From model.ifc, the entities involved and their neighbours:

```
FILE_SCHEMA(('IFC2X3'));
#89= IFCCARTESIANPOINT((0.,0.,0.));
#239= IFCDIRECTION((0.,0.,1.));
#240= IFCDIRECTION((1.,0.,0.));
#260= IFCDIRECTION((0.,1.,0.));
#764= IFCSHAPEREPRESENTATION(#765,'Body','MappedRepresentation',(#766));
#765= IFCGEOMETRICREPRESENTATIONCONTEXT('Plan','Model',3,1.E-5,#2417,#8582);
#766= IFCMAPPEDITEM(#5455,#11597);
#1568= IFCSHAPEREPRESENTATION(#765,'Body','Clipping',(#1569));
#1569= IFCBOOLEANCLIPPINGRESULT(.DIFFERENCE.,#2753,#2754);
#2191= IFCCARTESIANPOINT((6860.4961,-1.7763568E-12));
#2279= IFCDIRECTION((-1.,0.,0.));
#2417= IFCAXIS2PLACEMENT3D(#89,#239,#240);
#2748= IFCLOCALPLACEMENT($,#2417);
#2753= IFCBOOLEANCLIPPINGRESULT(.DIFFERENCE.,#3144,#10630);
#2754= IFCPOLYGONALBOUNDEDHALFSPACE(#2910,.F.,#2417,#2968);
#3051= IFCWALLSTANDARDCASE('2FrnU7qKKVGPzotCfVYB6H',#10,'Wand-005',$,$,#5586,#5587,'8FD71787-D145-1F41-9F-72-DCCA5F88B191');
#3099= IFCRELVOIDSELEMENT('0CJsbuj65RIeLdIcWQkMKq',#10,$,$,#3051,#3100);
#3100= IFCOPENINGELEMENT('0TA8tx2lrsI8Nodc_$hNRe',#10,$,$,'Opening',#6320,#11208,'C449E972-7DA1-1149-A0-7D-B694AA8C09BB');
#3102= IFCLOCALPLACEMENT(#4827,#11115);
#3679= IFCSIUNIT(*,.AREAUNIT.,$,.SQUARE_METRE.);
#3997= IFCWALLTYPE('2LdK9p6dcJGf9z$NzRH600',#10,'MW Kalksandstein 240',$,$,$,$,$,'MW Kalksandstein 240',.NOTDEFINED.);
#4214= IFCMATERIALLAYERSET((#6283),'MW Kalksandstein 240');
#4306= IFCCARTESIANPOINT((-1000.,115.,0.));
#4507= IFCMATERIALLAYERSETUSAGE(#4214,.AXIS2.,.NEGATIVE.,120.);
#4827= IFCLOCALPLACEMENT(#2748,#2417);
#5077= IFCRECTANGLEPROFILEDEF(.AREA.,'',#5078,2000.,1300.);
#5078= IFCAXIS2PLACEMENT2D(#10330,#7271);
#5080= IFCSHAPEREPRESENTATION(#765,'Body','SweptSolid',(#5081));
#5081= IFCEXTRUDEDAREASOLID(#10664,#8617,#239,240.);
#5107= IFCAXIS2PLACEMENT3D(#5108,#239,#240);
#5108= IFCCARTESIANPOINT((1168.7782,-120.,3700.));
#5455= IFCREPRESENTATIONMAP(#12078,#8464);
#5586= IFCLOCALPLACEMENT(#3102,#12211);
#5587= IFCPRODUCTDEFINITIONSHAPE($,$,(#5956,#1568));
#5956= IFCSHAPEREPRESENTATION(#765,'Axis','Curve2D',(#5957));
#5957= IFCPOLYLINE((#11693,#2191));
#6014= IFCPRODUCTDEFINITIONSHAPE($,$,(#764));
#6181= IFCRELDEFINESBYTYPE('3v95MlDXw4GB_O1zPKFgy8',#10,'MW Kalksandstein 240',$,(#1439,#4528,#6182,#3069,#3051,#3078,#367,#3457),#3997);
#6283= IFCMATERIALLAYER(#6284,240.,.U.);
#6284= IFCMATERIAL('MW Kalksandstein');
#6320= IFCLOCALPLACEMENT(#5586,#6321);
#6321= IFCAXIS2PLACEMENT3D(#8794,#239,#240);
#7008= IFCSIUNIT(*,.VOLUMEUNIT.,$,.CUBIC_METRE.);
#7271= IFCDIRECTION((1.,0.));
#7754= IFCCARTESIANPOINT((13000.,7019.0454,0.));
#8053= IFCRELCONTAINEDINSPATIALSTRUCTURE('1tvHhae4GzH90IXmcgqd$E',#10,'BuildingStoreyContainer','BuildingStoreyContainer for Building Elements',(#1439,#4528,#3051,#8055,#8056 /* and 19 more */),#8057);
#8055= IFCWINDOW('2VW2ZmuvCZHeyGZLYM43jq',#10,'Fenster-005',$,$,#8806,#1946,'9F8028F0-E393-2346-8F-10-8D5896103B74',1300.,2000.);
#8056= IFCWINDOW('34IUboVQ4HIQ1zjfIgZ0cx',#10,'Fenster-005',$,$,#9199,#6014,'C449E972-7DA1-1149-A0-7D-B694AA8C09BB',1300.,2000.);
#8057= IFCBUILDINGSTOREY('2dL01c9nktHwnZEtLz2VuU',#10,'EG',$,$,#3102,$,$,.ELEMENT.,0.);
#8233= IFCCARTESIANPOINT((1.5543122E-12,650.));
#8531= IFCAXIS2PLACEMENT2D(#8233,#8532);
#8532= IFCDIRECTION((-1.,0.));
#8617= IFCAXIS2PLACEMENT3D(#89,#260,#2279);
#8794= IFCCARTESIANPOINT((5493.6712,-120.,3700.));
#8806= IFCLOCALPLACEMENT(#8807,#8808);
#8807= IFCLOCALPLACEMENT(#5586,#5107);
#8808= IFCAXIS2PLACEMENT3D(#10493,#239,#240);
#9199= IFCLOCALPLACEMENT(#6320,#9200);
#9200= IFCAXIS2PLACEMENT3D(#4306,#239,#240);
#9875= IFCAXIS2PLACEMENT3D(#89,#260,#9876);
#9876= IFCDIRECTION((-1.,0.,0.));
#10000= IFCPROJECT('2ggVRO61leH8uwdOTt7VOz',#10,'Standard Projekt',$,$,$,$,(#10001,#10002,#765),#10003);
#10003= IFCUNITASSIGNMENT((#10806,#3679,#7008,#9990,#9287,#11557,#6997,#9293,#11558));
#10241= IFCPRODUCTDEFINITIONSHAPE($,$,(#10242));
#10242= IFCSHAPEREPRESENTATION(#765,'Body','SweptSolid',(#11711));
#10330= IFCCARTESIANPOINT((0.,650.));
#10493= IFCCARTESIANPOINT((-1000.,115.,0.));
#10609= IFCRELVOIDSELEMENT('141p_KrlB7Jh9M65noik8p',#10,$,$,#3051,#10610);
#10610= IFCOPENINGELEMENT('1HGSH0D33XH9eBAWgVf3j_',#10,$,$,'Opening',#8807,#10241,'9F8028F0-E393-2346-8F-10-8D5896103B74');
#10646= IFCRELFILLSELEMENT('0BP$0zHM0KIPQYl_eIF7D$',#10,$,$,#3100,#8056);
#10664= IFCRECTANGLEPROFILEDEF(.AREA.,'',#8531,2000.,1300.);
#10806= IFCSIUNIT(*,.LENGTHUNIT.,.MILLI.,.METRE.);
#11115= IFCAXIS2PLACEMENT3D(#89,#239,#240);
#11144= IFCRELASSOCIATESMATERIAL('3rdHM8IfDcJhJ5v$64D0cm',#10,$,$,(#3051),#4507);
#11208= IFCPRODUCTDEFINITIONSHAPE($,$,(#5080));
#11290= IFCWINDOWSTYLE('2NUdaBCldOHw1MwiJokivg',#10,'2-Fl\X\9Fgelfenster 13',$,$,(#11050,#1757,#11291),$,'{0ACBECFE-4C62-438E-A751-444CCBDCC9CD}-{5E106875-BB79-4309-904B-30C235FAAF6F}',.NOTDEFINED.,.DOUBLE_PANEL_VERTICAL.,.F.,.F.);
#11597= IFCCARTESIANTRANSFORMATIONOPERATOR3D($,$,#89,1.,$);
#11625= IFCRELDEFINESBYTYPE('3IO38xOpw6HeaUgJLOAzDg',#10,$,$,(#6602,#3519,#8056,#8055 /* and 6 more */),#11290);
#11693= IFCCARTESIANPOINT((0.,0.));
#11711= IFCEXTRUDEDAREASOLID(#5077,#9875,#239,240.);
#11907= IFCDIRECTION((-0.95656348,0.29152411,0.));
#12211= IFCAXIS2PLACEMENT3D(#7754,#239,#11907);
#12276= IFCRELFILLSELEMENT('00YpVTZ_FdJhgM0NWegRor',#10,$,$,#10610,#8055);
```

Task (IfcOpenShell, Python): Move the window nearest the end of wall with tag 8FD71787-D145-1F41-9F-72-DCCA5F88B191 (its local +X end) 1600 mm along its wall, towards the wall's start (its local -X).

```python
import ifcopenshell
import ifcopenshell.api.geometry
import ifcopenshell.util.placement
import ifcopenshell.util.unit

model = ifcopenshell.open("model.ifc")
unit_scale = ifcopenshell.util.unit.calculate_unit_scale(model)

window = model.by_id(8056)
opening = window.FillsVoids[0].RelatingOpeningElement
wall = opening.VoidsElements[0].RelatingBuildingElement

wall_matrix = ifcopenshell.util.placement.get_local_placement(wall.ObjectPlacement)
shift = wall_matrix[:3, 0] * -1.6 / unit_scale
before = ifcopenshell.util.placement.get_local_placement(window.ObjectPlacement)[:3, 3].copy()

# The window is placed relative to its opening, so it follows when the opening moves.
matrix = ifcopenshell.util.placement.get_local_placement(opening.ObjectPlacement)
matrix[:3, 3] += shift
ifcopenshell.api.geometry.edit_object_placement(
    model, product=opening, matrix=matrix, is_si=False, should_transform_children=True
)

after = ifcopenshell.util.placement.get_local_placement(window.ObjectPlacement)[:3, 3]
print("window moved by", (after - before).round(3) + 0.0)

model.write("model_rev.ifc")
```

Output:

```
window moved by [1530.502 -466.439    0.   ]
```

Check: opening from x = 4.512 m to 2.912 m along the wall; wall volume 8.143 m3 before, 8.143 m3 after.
